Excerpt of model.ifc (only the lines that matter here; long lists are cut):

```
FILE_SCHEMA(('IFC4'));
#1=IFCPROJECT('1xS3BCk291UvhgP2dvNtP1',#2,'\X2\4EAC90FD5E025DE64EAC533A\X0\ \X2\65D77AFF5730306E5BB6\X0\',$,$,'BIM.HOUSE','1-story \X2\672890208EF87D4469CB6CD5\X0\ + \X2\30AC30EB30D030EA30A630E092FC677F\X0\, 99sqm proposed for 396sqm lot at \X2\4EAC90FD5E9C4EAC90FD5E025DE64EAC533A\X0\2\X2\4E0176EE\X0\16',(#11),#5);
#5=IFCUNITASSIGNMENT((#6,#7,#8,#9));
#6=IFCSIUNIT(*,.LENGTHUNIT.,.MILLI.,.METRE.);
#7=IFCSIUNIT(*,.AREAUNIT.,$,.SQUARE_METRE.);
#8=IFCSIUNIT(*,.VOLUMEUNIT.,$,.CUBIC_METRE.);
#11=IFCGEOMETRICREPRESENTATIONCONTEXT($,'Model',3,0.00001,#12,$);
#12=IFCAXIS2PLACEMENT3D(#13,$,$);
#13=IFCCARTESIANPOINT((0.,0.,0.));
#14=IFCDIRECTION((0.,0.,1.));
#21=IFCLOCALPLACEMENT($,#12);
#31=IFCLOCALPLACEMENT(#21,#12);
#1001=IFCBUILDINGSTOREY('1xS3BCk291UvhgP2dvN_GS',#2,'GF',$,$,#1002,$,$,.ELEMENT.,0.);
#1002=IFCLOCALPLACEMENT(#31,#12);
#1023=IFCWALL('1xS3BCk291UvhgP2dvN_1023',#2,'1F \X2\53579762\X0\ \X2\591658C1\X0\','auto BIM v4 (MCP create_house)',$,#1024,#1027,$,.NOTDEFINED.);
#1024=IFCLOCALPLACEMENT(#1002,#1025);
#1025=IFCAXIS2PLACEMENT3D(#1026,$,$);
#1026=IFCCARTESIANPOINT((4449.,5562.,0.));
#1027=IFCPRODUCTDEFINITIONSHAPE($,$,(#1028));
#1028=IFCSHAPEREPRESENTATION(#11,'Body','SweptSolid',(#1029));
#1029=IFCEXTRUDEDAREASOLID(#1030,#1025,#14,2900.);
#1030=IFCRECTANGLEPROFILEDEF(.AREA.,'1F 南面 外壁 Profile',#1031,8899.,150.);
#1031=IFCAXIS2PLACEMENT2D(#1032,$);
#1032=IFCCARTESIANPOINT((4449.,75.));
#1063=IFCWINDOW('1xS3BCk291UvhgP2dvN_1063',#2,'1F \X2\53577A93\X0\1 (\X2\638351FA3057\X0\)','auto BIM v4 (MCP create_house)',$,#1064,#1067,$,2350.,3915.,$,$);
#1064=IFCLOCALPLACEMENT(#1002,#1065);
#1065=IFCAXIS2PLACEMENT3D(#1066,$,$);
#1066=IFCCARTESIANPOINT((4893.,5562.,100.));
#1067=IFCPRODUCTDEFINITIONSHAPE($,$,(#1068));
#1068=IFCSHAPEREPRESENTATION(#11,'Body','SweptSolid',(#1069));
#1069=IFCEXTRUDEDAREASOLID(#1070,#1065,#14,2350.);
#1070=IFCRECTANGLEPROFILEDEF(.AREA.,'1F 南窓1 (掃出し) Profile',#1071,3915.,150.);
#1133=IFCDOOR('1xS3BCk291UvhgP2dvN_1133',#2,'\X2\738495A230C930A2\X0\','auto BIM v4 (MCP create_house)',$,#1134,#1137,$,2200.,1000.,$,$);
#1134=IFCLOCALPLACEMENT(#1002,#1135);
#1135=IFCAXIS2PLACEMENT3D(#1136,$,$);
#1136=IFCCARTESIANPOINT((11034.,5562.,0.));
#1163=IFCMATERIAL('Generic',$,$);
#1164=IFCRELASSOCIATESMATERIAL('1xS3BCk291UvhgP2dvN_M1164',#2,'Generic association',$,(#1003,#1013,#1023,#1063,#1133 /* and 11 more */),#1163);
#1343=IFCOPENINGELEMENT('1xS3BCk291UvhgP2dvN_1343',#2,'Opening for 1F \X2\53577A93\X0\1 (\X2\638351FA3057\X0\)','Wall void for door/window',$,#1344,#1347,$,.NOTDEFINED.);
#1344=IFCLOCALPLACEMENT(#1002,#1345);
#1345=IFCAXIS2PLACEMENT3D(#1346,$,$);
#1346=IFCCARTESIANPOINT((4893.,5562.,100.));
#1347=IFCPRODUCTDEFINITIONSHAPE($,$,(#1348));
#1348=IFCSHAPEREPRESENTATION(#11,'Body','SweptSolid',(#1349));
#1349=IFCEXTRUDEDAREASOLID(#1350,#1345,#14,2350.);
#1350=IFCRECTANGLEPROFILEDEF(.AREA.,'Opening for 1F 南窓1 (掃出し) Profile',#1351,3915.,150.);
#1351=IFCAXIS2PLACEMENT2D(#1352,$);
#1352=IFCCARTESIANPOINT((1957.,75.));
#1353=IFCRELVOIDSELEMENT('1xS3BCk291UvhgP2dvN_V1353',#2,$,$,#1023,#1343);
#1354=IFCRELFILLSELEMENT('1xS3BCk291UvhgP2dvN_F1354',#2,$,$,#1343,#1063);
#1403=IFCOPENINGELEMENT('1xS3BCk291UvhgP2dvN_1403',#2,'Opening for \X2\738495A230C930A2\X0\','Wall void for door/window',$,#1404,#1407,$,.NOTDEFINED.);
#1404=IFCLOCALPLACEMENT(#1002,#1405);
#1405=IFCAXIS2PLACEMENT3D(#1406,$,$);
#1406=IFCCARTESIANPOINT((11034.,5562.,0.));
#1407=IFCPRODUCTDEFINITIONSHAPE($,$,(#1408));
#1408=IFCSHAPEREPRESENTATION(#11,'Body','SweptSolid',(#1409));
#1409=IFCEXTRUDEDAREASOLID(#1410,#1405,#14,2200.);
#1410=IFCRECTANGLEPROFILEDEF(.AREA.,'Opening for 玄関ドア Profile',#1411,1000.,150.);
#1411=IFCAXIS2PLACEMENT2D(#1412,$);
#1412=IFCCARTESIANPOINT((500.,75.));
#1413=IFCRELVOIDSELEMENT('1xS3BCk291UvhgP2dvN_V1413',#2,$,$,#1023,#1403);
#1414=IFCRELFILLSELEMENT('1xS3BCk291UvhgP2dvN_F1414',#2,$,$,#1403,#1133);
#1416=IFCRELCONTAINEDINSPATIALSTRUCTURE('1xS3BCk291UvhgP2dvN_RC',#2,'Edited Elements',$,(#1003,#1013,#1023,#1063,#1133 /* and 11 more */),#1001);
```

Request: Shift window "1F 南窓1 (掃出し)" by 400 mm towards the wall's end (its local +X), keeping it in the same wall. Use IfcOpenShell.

```python
import ifcopenshell
import ifcopenshell.api.geometry
import ifcopenshell.util.placement
import ifcopenshell.util.unit

model = ifcopenshell.open("model.ifc")
unit_scale = ifcopenshell.util.unit.calculate_unit_scale(model)

window = model.by_id(1063)
opening = window.FillsVoids[0].RelatingOpeningElement
wall = opening.VoidsElements[0].RelatingBuildingElement

wall_matrix = ifcopenshell.util.placement.get_local_placement(wall.ObjectPlacement)
shift = wall_matrix[:3, 0] * 0.4 / unit_scale
before = ifcopenshell.util.placement.get_local_placement(window.ObjectPlacement)[:3, 3].copy()

# The window is not placed relative to its opening, so move both.
for product in (opening, window):
    matrix = ifcopenshell.util.placement.get_local_placement(product.ObjectPlacement)
    matrix[:3, 3] += shift
    ifcopenshell.api.geometry.edit_object_placement(model, product=product, matrix=matrix, is_si=False)

after = ifcopenshell.util.placement.get_local_placement(window.ObjectPlacement)[:3, 3]
print("window moved by", (after - before).round(3) + 0.0)

model.write("model-out.ifc")
```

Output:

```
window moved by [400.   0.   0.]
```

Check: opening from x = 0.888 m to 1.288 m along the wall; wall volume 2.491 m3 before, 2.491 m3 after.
